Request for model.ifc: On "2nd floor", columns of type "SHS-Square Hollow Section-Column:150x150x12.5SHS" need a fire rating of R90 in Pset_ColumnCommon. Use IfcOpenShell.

First a look at what the model holds.

```python
import ifcopenshell
import ifcopenshell.util.element

model = ifcopenshell.open("model.ifc")
print(model.schema)
storey = next(s for s in model.by_type("IfcBuildingStorey") if s.Name == "2nd floor")
columns = [e for e in ifcopenshell.util.element.get_decomposition(storey) if e.is_a("IfcColumn")]
seen = {}
for e in columns:
    element_type = ifcopenshell.util.element.get_type(e)
    key = (element_type.Name if element_type != e and element_type else None, ifcopenshell.util.element.get_pset(e, "Pset_ColumnCommon", "FireRating"))
    seen[key] = seen.get(key, 0) + 1
for (name, value), count in sorted(seen.items(), key=str):
    print(count, "x", name, "|", value)
```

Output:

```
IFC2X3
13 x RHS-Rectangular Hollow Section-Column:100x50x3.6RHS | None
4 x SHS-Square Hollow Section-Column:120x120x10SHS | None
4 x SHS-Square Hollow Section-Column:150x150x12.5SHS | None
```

```python
import ifcopenshell
import ifcopenshell.api.pset
import ifcopenshell.util.element

model = ifcopenshell.open("model.ifc")

storey = next(s for s in model.by_type("IfcBuildingStorey") if s.Name == "2nd floor")
columns = [e for e in ifcopenshell.util.element.get_decomposition(storey) if e.is_a("IfcColumn")]

count = 0
for e in columns:
    element_type = ifcopenshell.util.element.get_type(e)
    if element_type in (None, e) or element_type.Name != "SHS-Square Hollow Section-Column:150x150x12.5SHS":
        continue
    # add_pset returns the element's existing set when there is one.
    pset = ifcopenshell.api.pset.add_pset(model, product=e, name="Pset_ColumnCommon")
    ifcopenshell.api.pset.edit_pset(model, pset=pset, properties={"FireRating": "R90"})
    count += 1

print(count, "columns updated")

model.write("model_rev.ifc")
```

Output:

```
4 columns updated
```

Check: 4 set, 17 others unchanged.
